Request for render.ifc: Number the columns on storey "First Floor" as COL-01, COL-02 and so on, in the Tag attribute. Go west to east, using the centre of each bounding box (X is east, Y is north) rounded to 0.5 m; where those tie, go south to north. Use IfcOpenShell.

First a look at what the model holds.

```python
import ifcopenshell
import ifcopenshell.util.element
import ifcopenshell.util.placement

model = ifcopenshell.open("render.ifc")
print(model.schema)
storey = next(s for s in model.by_type("IfcBuildingStorey") if s.Name == "First Floor")
columns = [e for e in ifcopenshell.util.element.get_decomposition(storey) if e.is_a("IfcColumn")]
for e in sorted(columns, key=lambda e: e.id()):
    origin = ifcopenshell.util.placement.get_local_placement(e.ObjectPlacement)[:3, 3]
    print(e.id(), e.Tag, e.Name, origin.round(2) + 0.0, sep=" | ")
```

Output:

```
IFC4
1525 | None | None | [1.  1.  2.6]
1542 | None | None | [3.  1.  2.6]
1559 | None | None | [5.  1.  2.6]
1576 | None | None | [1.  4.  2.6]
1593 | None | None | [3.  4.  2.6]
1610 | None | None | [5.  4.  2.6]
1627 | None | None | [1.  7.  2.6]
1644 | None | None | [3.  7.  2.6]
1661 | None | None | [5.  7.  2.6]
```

```python
import ifcopenshell
import ifcopenshell.geom
import ifcopenshell.util.element
import ifcopenshell.util.shape

model = ifcopenshell.open("render.ifc")
settings = ifcopenshell.geom.settings()
settings.set("use-world-coords", True)


def centre(element):
    shape = ifcopenshell.geom.create_shape(settings, element)
    return ifcopenshell.util.shape.get_bbox_centroid(shape.geometry)


storey = next(s for s in model.by_type("IfcBuildingStorey") if s.Name == "First Floor")
columns = [e for e in ifcopenshell.util.element.get_decomposition(storey) if e.is_a("IfcColumn")]

# Insertion points can sit at a corner or the storey origin, so sort by the geometry (in metres).
centres = {e: centre(e) for e in columns}
columns.sort(key=lambda e: (round(centres[e][0] / 0.5), centres[e][1]))

for i, e in enumerate(columns, start=1):
    number = f"COL-{i:02d}"
    e.Tag = number
    print(e.id(), number)

model.write("render_rev.ifc")
```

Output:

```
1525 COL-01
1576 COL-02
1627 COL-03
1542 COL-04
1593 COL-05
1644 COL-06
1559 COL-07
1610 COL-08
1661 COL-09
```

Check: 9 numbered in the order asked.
